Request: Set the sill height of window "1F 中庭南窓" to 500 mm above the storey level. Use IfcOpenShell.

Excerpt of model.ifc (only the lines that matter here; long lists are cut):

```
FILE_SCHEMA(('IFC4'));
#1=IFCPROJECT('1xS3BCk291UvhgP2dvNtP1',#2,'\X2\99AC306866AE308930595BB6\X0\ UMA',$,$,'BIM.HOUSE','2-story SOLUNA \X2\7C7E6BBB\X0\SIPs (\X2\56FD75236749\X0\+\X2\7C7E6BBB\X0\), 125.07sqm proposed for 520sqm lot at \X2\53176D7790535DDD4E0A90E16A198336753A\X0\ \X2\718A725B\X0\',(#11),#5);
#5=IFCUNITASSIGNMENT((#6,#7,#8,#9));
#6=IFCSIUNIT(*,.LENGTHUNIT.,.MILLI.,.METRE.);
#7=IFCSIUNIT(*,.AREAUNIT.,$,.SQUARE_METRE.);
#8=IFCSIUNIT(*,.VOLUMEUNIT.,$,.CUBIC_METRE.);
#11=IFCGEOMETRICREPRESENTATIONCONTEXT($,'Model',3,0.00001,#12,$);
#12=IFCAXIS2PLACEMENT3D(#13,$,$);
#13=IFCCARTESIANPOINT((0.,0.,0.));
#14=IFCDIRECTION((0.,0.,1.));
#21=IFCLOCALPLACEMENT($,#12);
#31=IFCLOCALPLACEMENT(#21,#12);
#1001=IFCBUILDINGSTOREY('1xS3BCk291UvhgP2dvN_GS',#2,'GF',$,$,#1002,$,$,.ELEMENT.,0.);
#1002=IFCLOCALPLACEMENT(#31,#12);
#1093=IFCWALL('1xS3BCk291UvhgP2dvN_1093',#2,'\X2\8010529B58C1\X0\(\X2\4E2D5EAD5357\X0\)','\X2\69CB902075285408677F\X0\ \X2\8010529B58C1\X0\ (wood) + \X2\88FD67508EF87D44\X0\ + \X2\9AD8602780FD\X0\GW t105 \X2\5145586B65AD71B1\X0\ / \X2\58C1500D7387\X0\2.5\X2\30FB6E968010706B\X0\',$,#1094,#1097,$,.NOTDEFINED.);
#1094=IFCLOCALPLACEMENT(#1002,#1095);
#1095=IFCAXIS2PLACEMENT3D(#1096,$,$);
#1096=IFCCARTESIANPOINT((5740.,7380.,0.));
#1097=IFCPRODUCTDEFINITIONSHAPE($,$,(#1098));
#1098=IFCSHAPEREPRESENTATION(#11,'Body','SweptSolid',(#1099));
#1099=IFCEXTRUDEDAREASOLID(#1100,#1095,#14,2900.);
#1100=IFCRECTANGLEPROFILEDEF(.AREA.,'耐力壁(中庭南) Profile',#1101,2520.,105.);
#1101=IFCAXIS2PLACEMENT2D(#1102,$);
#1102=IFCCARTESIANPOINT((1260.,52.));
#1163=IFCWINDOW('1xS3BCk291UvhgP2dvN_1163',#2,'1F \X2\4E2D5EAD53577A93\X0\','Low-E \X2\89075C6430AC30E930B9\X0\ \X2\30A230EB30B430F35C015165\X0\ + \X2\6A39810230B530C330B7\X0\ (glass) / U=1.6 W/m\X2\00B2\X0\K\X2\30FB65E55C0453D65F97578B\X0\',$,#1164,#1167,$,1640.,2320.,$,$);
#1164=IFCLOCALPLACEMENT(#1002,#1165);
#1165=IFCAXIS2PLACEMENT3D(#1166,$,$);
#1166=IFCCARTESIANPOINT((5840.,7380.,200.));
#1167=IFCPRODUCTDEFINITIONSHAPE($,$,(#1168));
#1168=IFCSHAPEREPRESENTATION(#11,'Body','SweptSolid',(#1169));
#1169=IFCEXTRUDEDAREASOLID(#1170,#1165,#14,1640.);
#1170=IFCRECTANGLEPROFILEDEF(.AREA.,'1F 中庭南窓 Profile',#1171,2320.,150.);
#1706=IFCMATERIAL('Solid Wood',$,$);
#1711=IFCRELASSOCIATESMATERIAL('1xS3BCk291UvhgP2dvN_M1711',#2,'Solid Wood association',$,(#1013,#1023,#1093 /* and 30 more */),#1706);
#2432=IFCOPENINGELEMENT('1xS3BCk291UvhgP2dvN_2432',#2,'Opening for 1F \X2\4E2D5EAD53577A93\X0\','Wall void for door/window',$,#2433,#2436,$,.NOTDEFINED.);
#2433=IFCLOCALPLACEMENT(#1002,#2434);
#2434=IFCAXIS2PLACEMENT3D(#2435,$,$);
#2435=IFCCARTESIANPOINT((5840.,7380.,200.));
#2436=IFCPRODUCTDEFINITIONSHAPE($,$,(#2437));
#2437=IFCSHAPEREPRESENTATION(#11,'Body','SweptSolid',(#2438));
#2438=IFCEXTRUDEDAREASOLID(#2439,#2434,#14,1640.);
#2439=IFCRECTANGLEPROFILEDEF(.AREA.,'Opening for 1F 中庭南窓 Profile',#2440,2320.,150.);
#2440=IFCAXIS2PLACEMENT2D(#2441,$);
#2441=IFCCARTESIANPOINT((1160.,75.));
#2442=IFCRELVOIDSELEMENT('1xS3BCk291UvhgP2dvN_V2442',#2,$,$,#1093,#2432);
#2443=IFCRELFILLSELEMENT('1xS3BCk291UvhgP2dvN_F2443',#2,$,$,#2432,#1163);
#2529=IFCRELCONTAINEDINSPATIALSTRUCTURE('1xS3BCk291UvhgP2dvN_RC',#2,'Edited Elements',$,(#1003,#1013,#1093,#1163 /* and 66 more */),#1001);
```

```python
import numpy as np
import ifcopenshell
import ifcopenshell.api.geometry
import ifcopenshell.geom
import ifcopenshell.util.element
import ifcopenshell.util.placement
import ifcopenshell.util.shape
import ifcopenshell.util.unit

model = ifcopenshell.open("model.ifc")
unit_scale = ifcopenshell.util.unit.calculate_unit_scale(model)

window = model.by_guid("1xS3BCk291UvhgP2dvN_1163")
opening = window.FillsVoids[0].RelatingOpeningElement
storey = ifcopenshell.util.element.get_container(window, ifc_class="IfcBuildingStorey")
level = ifcopenshell.util.placement.get_local_placement(storey.ObjectPlacement)[2, 3]

# The opening's origin need not be at the sill, so measure its lowest point.
shape = ifcopenshell.geom.create_shape(ifcopenshell.geom.settings(), opening)
bottom = ifcopenshell.util.shape.get_shape_bottom_elevation(shape, shape.geometry) / unit_scale
dz = level + 0.5 / unit_scale - bottom

shift = np.array([0.0, 0.0, dz])
# The window is not placed relative to its opening, so move both.
for product in (opening, window):
    matrix = ifcopenshell.util.placement.get_local_placement(product.ObjectPlacement)
    matrix[:3, 3] += shift
    ifcopenshell.api.geometry.edit_object_placement(model, product=product, matrix=matrix, is_si=False)

print(f"moved by {dz * unit_scale:+.3f} m")

model.write("model-out.ifc")
```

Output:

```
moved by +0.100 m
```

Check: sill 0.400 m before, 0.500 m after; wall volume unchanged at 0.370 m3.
